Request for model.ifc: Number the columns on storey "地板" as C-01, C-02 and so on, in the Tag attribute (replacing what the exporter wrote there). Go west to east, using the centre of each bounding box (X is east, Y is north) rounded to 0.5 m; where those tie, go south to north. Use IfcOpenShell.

First a look at what the model holds.

```python
import ifcopenshell
import ifcopenshell.util.element
import ifcopenshell.util.placement

model = ifcopenshell.open("model.ifc")
print(model.schema)
storey = next(s for s in model.by_type("IfcBuildingStorey") if s.Name == "地板")
columns = [e for e in ifcopenshell.util.element.get_decomposition(storey) if e.is_a("IfcColumn")]
for e in sorted(columns, key=lambda e: e.id()):
    origin = ifcopenshell.util.placement.get_local_placement(e.ObjectPlacement)[:3, 3]
    print(e.id(), e.Tag, e.Name, origin.round(2) + 0.0, sep=" | ")
```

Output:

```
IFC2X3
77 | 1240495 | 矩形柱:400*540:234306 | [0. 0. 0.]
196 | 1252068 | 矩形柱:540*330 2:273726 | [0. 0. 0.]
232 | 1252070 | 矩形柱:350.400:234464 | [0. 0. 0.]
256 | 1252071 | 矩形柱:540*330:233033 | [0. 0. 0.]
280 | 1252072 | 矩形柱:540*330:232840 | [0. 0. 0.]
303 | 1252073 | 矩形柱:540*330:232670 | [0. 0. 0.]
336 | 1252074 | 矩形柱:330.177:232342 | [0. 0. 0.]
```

```python
import ifcopenshell
import ifcopenshell.geom
import ifcopenshell.util.element
import ifcopenshell.util.shape

model = ifcopenshell.open("model.ifc")
settings = ifcopenshell.geom.settings()
settings.set("use-world-coords", True)


def centre(element):
    shape = ifcopenshell.geom.create_shape(settings, element)
    return ifcopenshell.util.shape.get_bbox_centroid(shape.geometry)


storey = next(s for s in model.by_type("IfcBuildingStorey") if s.Name == "地板")
columns = [e for e in ifcopenshell.util.element.get_decomposition(storey) if e.is_a("IfcColumn")]

# Insertion points can sit at a corner or the storey origin, so sort by the geometry (in metres).
centres = {e: centre(e) for e in columns}
columns.sort(key=lambda e: (round(centres[e][0] / 0.5), centres[e][1]))

for i, e in enumerate(columns, start=1):
    number = f"C-{i:02d}"
    e.Tag = number
    print(e.id(), number)

model.write("model_updated.ifc")
```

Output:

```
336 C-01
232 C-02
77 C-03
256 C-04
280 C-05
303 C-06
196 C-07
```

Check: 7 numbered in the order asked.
